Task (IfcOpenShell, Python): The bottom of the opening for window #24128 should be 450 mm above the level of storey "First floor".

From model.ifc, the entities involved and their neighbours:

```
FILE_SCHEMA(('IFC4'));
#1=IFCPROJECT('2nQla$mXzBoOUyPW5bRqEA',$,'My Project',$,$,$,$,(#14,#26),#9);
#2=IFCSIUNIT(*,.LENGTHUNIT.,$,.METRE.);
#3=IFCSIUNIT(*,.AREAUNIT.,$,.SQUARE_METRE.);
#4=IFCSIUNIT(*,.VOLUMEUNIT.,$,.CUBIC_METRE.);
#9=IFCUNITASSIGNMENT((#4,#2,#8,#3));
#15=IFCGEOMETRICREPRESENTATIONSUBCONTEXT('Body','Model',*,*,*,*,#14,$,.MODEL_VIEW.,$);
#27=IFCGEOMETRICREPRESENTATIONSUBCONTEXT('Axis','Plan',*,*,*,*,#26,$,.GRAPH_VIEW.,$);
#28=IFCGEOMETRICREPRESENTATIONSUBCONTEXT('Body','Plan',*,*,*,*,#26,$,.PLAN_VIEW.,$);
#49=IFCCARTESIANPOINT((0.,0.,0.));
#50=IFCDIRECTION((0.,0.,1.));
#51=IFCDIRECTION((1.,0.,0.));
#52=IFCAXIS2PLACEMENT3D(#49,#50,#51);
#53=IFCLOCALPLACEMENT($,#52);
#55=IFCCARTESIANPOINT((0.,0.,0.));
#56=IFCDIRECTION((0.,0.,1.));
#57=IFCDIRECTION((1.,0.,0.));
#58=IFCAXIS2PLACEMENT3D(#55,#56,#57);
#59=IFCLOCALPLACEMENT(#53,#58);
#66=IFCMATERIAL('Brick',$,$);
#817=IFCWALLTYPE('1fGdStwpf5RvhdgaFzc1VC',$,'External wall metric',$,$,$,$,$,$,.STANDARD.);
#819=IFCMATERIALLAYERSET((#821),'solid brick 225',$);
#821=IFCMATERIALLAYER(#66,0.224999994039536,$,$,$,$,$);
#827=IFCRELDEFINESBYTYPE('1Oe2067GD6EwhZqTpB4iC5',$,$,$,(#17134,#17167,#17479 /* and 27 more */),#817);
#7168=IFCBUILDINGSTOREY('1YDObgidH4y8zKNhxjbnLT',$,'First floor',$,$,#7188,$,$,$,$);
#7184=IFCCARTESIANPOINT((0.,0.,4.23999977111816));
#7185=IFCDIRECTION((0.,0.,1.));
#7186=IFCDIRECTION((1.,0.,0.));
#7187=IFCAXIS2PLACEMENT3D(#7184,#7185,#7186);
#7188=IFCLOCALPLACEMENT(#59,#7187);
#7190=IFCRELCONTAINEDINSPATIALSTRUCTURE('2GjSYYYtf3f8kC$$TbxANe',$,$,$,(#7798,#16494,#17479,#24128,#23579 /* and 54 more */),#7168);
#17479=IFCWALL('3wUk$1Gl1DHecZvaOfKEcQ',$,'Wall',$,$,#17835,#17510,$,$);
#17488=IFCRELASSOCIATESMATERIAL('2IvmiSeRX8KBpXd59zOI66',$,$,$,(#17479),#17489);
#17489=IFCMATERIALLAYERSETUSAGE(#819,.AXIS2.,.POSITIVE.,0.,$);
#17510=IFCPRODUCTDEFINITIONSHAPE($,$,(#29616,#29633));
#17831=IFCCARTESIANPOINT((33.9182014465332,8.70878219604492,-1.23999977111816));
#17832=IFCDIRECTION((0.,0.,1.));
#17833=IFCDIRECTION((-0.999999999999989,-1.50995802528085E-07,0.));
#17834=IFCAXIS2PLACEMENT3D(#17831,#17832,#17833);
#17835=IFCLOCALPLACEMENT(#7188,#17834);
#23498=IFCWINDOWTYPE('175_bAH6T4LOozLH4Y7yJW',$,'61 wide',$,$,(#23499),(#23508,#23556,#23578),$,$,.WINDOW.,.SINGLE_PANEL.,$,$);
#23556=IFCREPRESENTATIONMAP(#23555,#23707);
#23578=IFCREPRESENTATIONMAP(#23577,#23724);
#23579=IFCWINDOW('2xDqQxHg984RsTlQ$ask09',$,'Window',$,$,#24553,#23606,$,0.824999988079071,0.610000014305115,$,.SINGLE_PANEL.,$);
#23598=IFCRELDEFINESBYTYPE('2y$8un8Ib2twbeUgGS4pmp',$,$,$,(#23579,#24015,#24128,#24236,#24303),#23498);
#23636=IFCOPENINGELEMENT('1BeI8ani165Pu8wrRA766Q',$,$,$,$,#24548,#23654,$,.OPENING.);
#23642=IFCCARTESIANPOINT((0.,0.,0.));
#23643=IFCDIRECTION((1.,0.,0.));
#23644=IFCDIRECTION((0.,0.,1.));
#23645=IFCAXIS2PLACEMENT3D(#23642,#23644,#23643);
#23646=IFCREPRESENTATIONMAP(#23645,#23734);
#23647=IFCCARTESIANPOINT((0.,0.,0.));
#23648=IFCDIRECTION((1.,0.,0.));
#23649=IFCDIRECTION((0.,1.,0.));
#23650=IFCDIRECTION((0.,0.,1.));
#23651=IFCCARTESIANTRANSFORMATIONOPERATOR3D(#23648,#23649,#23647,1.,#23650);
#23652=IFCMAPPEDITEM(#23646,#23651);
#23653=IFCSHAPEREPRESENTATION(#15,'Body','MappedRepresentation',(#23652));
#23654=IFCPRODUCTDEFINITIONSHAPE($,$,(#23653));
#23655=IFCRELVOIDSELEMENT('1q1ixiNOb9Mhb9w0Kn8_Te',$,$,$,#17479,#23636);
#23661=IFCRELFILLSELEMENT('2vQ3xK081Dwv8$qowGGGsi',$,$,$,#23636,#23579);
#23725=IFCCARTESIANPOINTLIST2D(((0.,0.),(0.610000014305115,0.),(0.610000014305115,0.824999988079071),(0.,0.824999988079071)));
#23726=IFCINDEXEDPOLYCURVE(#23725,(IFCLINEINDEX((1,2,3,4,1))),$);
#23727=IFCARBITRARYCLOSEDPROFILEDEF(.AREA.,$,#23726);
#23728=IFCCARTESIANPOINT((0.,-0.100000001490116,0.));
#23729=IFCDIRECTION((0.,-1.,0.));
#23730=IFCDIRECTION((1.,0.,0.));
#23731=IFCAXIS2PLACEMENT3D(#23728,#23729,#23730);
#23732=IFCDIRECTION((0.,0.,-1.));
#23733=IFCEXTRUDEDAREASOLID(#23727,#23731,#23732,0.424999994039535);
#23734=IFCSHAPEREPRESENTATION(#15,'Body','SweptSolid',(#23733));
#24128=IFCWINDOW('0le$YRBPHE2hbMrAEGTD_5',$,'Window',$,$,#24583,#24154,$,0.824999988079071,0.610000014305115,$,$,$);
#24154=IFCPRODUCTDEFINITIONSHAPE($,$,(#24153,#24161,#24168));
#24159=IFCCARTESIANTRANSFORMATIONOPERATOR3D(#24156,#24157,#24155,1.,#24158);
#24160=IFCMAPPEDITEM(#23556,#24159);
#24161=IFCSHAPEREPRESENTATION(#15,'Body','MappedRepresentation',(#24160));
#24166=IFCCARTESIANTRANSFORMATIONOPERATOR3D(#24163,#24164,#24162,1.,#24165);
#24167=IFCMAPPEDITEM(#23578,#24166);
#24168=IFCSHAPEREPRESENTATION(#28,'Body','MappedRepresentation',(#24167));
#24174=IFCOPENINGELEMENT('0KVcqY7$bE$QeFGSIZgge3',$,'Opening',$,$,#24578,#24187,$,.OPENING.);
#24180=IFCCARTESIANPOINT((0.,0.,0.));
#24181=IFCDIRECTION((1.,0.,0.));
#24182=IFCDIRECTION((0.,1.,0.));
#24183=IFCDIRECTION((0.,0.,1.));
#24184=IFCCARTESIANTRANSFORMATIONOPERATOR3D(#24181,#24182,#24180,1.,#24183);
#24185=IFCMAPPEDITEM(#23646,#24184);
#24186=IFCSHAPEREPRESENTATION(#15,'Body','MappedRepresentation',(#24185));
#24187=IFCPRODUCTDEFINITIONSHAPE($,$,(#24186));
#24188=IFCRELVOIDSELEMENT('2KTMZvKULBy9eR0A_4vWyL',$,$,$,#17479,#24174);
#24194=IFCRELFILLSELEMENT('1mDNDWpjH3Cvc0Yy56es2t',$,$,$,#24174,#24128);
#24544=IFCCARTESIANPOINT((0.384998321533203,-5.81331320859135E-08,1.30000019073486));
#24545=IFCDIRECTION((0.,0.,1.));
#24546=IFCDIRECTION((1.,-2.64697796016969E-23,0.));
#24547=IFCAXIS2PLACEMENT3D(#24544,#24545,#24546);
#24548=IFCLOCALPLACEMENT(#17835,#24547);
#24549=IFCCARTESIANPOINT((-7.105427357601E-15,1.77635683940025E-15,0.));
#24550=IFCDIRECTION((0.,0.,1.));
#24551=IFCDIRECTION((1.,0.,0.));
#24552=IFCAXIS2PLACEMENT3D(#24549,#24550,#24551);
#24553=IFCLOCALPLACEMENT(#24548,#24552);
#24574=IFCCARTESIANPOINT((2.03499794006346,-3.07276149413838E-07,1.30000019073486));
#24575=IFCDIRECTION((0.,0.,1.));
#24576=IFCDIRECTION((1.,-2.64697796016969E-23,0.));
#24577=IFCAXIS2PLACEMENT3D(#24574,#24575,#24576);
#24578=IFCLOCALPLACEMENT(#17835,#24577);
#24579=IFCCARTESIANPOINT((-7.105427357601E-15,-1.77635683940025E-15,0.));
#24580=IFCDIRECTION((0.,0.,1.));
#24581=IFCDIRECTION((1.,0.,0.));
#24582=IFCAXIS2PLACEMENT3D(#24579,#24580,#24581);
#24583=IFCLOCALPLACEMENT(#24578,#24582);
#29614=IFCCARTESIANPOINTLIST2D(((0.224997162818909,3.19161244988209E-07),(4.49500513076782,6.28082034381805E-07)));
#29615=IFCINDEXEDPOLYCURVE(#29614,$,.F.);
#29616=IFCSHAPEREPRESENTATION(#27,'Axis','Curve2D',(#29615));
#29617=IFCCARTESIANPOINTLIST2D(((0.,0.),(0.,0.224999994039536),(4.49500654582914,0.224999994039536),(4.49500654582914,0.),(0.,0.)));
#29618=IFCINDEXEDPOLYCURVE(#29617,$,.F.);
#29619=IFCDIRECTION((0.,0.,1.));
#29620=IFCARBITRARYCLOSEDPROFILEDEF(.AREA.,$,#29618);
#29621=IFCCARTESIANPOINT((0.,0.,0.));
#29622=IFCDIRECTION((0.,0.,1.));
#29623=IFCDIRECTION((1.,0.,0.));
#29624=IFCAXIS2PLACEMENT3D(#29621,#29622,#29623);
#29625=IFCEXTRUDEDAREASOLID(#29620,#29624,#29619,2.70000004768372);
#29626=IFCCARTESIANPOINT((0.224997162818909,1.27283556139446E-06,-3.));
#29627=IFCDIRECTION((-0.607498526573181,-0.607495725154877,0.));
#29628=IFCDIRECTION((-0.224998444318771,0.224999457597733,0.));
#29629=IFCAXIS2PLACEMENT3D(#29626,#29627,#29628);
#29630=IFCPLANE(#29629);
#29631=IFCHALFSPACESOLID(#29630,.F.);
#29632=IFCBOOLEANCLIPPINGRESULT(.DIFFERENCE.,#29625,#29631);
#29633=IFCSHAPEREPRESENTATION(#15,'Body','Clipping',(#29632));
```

```python
import numpy as np
import ifcopenshell
import ifcopenshell.api.geometry
import ifcopenshell.geom
import ifcopenshell.util.element
import ifcopenshell.util.placement
import ifcopenshell.util.shape
import ifcopenshell.util.unit

model = ifcopenshell.open("model.ifc")
unit_scale = ifcopenshell.util.unit.calculate_unit_scale(model)

window = model.by_id(24128)
opening = window.FillsVoids[0].RelatingOpeningElement
storey = ifcopenshell.util.element.get_container(window, ifc_class="IfcBuildingStorey")
level = ifcopenshell.util.placement.get_local_placement(storey.ObjectPlacement)[2, 3]

# The opening's origin need not be at the sill, so measure its lowest point.
shape = ifcopenshell.geom.create_shape(ifcopenshell.geom.settings(), opening)
bottom = ifcopenshell.util.shape.get_shape_bottom_elevation(shape, shape.geometry) / unit_scale
dz = level + 0.45 / unit_scale - bottom

shift = np.array([0.0, 0.0, dz])
# The window is placed relative to its opening, so it follows when the opening moves.
matrix = ifcopenshell.util.placement.get_local_placement(opening.ObjectPlacement)
matrix[:3, 3] += shift
ifcopenshell.api.geometry.edit_object_placement(
    model, product=opening, matrix=matrix, is_si=False, should_transform_children=True
)

print(f"moved by {dz * unit_scale:+.3f} m")

model.write("model-out.ifc")
```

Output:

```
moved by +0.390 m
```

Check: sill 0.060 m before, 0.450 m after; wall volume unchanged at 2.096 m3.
